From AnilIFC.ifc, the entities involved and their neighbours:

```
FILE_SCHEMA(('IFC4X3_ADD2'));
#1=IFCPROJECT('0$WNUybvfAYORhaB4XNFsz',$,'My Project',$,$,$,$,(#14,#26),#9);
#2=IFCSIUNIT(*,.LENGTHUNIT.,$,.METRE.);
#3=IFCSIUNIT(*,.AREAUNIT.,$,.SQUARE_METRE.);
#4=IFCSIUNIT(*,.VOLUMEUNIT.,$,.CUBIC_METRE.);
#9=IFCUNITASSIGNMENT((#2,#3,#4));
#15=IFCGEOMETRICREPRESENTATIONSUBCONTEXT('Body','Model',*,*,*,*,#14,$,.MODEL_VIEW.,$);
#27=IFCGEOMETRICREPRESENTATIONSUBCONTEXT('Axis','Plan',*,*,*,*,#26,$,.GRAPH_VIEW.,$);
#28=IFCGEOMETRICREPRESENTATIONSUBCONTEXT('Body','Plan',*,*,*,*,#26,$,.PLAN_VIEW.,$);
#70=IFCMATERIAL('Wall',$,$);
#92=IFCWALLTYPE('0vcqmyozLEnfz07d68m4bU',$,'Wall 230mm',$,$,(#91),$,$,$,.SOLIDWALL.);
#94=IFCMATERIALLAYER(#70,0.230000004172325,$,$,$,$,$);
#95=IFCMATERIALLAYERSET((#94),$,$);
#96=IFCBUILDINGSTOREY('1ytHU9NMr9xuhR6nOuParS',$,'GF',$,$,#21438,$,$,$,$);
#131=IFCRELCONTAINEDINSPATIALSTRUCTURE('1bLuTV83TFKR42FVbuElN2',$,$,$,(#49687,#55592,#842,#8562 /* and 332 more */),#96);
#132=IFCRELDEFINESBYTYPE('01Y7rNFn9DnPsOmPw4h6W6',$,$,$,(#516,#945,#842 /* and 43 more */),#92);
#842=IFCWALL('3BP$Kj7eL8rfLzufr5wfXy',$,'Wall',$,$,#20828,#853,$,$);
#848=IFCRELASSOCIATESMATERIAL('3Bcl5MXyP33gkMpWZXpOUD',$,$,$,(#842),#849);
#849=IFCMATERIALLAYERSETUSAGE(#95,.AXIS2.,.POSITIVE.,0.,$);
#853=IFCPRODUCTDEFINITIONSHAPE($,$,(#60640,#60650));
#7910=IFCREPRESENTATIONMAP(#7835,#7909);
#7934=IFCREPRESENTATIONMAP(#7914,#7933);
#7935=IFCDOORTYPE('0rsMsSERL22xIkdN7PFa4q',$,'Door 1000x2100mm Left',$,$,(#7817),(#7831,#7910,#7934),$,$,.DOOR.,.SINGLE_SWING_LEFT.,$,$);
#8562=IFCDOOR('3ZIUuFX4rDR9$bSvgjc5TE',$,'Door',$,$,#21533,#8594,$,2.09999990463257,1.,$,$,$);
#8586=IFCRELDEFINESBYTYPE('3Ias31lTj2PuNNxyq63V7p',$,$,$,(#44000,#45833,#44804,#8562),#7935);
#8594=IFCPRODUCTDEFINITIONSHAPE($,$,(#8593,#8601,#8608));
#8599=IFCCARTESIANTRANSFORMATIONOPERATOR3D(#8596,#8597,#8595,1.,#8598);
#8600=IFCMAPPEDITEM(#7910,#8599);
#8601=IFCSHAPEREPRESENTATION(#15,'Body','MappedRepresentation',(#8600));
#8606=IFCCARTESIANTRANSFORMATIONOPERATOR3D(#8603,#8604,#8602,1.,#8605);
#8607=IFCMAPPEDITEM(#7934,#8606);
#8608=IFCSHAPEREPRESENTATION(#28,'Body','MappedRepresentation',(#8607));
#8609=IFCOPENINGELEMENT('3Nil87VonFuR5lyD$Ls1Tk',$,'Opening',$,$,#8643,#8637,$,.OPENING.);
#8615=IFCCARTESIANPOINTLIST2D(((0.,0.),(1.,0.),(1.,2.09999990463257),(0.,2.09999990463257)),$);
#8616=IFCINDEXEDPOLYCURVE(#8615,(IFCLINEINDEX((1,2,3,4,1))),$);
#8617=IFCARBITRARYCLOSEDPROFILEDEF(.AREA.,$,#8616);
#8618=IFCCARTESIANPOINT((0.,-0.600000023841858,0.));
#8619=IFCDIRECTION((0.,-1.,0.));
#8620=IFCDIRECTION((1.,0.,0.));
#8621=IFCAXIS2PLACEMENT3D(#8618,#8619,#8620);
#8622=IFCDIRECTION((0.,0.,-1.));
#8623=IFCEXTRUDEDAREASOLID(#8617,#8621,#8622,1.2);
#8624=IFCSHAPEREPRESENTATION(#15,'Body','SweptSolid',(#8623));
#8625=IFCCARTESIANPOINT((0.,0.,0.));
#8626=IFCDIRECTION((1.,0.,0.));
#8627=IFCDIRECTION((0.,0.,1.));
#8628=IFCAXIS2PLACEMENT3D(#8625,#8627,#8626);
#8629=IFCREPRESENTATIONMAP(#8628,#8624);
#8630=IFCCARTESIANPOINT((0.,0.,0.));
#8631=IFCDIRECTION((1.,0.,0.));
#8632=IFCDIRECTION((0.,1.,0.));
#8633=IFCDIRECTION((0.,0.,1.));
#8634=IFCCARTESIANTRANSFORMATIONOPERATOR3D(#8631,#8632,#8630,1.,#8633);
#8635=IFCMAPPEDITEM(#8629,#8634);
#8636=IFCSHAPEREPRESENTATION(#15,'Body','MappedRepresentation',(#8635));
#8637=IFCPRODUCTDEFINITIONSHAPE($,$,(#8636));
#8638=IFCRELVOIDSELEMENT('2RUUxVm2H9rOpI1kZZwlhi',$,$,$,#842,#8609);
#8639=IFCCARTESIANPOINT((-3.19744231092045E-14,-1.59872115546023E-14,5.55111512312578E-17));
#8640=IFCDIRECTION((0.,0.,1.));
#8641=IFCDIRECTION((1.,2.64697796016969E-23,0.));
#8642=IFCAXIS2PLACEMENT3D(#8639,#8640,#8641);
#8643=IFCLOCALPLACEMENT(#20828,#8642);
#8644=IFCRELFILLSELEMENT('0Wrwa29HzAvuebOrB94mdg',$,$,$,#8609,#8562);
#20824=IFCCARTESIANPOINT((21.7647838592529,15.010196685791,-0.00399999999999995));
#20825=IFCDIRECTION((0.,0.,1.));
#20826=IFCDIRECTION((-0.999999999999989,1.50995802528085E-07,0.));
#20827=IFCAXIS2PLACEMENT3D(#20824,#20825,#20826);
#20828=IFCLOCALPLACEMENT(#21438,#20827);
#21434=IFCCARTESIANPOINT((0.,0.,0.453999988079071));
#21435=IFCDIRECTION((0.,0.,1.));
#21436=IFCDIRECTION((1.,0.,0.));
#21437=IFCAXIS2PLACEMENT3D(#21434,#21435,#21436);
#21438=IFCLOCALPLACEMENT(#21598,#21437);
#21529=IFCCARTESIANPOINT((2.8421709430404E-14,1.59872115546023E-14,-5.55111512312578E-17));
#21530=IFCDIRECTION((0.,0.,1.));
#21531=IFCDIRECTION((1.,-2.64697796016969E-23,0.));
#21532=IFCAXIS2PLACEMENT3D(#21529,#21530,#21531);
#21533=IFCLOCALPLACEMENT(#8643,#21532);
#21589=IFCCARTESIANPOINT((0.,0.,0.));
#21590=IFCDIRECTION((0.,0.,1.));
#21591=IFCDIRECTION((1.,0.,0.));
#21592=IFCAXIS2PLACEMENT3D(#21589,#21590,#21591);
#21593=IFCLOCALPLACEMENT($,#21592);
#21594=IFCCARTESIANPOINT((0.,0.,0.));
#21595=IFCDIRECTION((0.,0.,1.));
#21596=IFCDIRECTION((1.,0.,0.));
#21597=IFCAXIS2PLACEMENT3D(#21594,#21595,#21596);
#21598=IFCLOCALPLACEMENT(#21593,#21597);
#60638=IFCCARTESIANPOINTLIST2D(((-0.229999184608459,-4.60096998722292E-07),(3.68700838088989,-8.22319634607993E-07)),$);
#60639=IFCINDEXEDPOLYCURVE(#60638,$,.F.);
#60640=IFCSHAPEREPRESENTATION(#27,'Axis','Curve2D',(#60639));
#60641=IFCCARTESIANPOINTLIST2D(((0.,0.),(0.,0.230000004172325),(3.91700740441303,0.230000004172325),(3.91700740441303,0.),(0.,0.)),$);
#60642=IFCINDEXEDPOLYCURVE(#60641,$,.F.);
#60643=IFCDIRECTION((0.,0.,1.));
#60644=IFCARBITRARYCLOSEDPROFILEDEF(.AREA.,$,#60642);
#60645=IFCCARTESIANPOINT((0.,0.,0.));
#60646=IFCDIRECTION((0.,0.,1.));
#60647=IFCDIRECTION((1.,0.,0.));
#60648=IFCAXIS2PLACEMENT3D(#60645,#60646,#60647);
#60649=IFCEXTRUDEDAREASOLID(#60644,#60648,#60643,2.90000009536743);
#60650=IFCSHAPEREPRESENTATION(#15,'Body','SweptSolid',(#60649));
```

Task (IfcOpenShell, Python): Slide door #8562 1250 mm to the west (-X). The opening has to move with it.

```python
import ifcopenshell
import ifcopenshell.api.geometry
import ifcopenshell.util.placement

model = ifcopenshell.open("AnilIFC.ifc")

door = model.by_id(8562)
opening = door.FillsVoids[0].RelatingOpeningElement
wall = opening.VoidsElements[0].RelatingBuildingElement

wall_matrix = ifcopenshell.util.placement.get_local_placement(wall.ObjectPlacement)
shift = wall_matrix[:3, 0] * 1.25
before = ifcopenshell.util.placement.get_local_placement(door.ObjectPlacement)[:3, 3].copy()

# The door is placed relative to its opening, so it follows when the opening moves.
matrix = ifcopenshell.util.placement.get_local_placement(opening.ObjectPlacement)
matrix[:3, 3] += shift
ifcopenshell.api.geometry.edit_object_placement(
    model, product=opening, matrix=matrix, is_si=False, should_transform_children=True
)

after = ifcopenshell.util.placement.get_local_placement(door.ObjectPlacement)[:3, 3]
print("door moved by", (after - before).round(3) + 0.0)

model.write("AnilIFC-out.ifc")
```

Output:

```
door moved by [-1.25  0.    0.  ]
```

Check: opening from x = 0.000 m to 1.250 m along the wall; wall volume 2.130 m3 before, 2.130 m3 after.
